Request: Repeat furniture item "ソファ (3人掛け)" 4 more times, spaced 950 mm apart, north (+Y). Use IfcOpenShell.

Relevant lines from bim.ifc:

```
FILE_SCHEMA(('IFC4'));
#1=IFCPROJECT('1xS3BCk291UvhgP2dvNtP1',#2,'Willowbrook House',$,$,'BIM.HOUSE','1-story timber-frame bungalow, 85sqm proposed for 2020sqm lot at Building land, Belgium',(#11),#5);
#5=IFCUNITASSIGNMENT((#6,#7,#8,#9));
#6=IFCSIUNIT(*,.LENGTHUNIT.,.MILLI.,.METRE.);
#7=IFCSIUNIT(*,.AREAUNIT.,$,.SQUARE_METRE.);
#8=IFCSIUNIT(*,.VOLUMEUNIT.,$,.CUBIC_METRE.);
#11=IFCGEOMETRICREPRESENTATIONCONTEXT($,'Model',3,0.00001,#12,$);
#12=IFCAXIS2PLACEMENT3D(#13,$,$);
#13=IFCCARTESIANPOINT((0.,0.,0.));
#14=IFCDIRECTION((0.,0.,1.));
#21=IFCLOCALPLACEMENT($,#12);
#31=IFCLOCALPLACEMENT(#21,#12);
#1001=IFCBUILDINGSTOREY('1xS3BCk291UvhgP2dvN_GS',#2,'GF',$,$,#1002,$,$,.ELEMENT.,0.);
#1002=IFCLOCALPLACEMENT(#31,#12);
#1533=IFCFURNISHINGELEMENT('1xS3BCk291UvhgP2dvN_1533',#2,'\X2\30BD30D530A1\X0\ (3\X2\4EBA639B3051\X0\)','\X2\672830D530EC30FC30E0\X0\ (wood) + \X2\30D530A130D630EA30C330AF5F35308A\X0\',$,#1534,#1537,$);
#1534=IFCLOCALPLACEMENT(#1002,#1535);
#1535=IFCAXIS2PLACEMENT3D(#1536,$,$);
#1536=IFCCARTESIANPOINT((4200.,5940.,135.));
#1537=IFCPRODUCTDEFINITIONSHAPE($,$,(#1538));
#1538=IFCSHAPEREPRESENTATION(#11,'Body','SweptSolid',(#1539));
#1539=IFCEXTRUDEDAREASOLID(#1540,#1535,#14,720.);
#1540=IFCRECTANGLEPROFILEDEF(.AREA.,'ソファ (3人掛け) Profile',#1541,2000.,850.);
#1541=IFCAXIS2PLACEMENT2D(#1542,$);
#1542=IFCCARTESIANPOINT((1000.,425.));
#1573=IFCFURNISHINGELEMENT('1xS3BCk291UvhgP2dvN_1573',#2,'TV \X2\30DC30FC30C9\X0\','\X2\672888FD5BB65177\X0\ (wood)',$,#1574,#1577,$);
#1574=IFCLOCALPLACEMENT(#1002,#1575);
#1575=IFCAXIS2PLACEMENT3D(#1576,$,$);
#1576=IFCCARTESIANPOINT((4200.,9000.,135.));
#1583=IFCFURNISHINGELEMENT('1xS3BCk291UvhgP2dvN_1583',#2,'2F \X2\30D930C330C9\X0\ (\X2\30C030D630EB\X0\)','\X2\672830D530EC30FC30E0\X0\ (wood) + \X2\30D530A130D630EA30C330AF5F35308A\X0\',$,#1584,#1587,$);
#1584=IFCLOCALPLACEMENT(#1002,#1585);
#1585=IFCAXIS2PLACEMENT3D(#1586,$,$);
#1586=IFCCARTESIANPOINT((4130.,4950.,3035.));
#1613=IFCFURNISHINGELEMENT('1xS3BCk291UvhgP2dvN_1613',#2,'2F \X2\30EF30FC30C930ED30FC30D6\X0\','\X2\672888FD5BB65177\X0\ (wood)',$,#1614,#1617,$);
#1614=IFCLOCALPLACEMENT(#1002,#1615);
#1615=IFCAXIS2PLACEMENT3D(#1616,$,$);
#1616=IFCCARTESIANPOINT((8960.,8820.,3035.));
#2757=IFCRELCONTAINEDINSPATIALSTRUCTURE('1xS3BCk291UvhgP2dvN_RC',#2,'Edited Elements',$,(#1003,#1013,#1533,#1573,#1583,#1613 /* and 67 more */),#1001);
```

```python
import numpy as np
import ifcopenshell
import ifcopenshell.api.geometry
import ifcopenshell.api.root
import ifcopenshell.util.element
import ifcopenshell.util.placement
import ifcopenshell.util.unit

model = ifcopenshell.open("bim.ifc")
unit_scale = ifcopenshell.util.unit.calculate_unit_scale(model)


def reuse_history(source, copy):
    """copy_class also copies each property set's owner history, people and application; keep the originals."""
    for rel in copy.IsDefinedBy:
        if rel.is_a("IfcRelDefinesByProperties") and (history := rel.RelatingPropertyDefinition.OwnerHistory):
            rel.RelatingPropertyDefinition.OwnerHistory = source.OwnerHistory
            ifcopenshell.util.element.remove_deep2(model, history)


source = model.by_guid("1xS3BCk291UvhgP2dvN_1533")
base = ifcopenshell.util.placement.get_local_placement(source.ObjectPlacement)
step = np.array([0.0, 1.0, 0.0]) * 0.95 / unit_scale

for i in range(1, 5):
    copy = ifcopenshell.api.root.copy_class(model, product=source)
    copy.Representation = ifcopenshell.util.element.copy_deep(
        model, source.Representation, exclude=["IfcGeometricRepresentationContext", "IfcRepresentationMap"]
    )
    reuse_history(source, copy)
    matrix = base.copy()
    matrix[:3, 3] += i * step
    print("added at", matrix[:3, 3].round(3) + 0.0)
    ifcopenshell.api.geometry.edit_object_placement(model, product=copy, matrix=matrix, is_si=False)

model.write("bim_updated.ifc")
```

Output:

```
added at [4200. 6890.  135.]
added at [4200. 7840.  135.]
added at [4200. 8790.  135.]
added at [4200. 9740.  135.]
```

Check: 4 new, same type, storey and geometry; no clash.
